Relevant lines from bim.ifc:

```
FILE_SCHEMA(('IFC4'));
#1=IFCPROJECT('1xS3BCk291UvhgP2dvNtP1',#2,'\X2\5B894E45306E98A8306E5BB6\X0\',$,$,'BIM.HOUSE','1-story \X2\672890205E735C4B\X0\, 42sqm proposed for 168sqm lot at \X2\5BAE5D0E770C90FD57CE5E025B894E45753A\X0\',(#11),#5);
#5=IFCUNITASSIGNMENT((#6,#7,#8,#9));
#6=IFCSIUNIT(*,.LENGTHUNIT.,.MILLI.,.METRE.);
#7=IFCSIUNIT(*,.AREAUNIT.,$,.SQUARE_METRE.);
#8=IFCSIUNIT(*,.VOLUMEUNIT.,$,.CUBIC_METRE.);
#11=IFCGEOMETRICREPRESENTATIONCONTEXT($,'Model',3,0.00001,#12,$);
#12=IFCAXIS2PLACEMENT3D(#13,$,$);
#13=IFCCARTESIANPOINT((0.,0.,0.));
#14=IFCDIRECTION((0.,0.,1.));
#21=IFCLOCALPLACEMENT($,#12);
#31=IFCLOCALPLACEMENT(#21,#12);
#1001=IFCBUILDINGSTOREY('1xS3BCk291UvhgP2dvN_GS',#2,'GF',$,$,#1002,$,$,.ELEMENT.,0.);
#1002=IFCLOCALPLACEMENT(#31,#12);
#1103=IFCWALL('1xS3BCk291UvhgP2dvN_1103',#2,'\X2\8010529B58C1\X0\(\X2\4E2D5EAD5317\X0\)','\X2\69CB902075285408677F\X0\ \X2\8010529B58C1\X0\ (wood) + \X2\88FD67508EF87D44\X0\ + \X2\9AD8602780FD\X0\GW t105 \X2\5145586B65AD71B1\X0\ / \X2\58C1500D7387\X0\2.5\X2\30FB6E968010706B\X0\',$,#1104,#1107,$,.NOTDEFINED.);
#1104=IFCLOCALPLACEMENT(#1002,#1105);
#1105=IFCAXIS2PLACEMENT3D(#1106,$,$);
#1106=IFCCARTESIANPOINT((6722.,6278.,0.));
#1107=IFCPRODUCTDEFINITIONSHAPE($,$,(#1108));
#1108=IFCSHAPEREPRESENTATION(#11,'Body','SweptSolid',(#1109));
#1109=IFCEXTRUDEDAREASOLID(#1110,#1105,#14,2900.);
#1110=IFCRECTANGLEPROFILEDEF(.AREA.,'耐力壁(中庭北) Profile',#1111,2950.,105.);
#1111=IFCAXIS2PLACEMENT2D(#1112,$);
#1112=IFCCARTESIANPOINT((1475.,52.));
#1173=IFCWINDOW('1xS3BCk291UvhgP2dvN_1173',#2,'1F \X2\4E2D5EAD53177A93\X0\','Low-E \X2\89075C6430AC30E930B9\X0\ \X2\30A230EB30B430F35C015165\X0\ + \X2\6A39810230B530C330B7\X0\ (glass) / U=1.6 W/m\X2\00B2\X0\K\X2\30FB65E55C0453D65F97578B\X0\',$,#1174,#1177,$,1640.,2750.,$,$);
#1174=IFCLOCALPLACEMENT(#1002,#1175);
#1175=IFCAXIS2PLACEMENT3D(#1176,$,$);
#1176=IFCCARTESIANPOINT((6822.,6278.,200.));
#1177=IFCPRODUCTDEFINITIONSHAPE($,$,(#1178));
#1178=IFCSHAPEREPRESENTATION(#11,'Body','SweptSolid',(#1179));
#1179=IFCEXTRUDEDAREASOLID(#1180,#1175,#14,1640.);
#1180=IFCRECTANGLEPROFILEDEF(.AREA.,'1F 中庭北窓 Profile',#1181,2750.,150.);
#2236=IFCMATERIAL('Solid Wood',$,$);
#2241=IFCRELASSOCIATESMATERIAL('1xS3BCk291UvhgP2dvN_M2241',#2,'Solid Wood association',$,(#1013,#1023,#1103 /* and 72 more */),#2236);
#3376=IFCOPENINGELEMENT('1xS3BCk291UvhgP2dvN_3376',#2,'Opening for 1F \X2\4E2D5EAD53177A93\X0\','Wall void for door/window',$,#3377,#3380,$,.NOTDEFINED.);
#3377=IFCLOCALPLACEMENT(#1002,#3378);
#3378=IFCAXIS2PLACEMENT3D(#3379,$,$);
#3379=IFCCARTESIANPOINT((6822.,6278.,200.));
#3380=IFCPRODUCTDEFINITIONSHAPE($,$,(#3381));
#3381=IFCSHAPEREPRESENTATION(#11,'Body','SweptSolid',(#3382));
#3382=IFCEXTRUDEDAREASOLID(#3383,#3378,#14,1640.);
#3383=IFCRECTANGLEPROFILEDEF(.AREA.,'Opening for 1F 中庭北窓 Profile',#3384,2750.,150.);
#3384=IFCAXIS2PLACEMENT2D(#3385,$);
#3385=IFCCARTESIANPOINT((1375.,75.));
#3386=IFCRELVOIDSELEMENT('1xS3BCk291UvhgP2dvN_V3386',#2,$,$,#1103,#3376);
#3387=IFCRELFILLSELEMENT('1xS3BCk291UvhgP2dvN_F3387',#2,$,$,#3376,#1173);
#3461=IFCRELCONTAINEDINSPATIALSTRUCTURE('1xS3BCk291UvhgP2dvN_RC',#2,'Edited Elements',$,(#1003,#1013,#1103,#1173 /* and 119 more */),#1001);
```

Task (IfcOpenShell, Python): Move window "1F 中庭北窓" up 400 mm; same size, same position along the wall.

```python
import numpy as np
import ifcopenshell
import ifcopenshell.api.geometry
import ifcopenshell.util.placement
import ifcopenshell.util.unit

model = ifcopenshell.open("bim.ifc")
unit_scale = ifcopenshell.util.unit.calculate_unit_scale(model)

window = model.by_guid("1xS3BCk291UvhgP2dvN_1173")
opening = window.FillsVoids[0].RelatingOpeningElement
dz = 400.0

shift = np.array([0.0, 0.0, dz])
# The window is not placed relative to its opening, so move both.
for product in (opening, window):
    matrix = ifcopenshell.util.placement.get_local_placement(product.ObjectPlacement)
    matrix[:3, 3] += shift
    ifcopenshell.api.geometry.edit_object_placement(model, product=product, matrix=matrix, is_si=False)

print(f"moved by {dz * unit_scale:+.3f} m")

model.write("bim_updated.ifc")
```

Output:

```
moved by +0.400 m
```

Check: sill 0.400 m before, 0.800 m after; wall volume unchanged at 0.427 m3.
